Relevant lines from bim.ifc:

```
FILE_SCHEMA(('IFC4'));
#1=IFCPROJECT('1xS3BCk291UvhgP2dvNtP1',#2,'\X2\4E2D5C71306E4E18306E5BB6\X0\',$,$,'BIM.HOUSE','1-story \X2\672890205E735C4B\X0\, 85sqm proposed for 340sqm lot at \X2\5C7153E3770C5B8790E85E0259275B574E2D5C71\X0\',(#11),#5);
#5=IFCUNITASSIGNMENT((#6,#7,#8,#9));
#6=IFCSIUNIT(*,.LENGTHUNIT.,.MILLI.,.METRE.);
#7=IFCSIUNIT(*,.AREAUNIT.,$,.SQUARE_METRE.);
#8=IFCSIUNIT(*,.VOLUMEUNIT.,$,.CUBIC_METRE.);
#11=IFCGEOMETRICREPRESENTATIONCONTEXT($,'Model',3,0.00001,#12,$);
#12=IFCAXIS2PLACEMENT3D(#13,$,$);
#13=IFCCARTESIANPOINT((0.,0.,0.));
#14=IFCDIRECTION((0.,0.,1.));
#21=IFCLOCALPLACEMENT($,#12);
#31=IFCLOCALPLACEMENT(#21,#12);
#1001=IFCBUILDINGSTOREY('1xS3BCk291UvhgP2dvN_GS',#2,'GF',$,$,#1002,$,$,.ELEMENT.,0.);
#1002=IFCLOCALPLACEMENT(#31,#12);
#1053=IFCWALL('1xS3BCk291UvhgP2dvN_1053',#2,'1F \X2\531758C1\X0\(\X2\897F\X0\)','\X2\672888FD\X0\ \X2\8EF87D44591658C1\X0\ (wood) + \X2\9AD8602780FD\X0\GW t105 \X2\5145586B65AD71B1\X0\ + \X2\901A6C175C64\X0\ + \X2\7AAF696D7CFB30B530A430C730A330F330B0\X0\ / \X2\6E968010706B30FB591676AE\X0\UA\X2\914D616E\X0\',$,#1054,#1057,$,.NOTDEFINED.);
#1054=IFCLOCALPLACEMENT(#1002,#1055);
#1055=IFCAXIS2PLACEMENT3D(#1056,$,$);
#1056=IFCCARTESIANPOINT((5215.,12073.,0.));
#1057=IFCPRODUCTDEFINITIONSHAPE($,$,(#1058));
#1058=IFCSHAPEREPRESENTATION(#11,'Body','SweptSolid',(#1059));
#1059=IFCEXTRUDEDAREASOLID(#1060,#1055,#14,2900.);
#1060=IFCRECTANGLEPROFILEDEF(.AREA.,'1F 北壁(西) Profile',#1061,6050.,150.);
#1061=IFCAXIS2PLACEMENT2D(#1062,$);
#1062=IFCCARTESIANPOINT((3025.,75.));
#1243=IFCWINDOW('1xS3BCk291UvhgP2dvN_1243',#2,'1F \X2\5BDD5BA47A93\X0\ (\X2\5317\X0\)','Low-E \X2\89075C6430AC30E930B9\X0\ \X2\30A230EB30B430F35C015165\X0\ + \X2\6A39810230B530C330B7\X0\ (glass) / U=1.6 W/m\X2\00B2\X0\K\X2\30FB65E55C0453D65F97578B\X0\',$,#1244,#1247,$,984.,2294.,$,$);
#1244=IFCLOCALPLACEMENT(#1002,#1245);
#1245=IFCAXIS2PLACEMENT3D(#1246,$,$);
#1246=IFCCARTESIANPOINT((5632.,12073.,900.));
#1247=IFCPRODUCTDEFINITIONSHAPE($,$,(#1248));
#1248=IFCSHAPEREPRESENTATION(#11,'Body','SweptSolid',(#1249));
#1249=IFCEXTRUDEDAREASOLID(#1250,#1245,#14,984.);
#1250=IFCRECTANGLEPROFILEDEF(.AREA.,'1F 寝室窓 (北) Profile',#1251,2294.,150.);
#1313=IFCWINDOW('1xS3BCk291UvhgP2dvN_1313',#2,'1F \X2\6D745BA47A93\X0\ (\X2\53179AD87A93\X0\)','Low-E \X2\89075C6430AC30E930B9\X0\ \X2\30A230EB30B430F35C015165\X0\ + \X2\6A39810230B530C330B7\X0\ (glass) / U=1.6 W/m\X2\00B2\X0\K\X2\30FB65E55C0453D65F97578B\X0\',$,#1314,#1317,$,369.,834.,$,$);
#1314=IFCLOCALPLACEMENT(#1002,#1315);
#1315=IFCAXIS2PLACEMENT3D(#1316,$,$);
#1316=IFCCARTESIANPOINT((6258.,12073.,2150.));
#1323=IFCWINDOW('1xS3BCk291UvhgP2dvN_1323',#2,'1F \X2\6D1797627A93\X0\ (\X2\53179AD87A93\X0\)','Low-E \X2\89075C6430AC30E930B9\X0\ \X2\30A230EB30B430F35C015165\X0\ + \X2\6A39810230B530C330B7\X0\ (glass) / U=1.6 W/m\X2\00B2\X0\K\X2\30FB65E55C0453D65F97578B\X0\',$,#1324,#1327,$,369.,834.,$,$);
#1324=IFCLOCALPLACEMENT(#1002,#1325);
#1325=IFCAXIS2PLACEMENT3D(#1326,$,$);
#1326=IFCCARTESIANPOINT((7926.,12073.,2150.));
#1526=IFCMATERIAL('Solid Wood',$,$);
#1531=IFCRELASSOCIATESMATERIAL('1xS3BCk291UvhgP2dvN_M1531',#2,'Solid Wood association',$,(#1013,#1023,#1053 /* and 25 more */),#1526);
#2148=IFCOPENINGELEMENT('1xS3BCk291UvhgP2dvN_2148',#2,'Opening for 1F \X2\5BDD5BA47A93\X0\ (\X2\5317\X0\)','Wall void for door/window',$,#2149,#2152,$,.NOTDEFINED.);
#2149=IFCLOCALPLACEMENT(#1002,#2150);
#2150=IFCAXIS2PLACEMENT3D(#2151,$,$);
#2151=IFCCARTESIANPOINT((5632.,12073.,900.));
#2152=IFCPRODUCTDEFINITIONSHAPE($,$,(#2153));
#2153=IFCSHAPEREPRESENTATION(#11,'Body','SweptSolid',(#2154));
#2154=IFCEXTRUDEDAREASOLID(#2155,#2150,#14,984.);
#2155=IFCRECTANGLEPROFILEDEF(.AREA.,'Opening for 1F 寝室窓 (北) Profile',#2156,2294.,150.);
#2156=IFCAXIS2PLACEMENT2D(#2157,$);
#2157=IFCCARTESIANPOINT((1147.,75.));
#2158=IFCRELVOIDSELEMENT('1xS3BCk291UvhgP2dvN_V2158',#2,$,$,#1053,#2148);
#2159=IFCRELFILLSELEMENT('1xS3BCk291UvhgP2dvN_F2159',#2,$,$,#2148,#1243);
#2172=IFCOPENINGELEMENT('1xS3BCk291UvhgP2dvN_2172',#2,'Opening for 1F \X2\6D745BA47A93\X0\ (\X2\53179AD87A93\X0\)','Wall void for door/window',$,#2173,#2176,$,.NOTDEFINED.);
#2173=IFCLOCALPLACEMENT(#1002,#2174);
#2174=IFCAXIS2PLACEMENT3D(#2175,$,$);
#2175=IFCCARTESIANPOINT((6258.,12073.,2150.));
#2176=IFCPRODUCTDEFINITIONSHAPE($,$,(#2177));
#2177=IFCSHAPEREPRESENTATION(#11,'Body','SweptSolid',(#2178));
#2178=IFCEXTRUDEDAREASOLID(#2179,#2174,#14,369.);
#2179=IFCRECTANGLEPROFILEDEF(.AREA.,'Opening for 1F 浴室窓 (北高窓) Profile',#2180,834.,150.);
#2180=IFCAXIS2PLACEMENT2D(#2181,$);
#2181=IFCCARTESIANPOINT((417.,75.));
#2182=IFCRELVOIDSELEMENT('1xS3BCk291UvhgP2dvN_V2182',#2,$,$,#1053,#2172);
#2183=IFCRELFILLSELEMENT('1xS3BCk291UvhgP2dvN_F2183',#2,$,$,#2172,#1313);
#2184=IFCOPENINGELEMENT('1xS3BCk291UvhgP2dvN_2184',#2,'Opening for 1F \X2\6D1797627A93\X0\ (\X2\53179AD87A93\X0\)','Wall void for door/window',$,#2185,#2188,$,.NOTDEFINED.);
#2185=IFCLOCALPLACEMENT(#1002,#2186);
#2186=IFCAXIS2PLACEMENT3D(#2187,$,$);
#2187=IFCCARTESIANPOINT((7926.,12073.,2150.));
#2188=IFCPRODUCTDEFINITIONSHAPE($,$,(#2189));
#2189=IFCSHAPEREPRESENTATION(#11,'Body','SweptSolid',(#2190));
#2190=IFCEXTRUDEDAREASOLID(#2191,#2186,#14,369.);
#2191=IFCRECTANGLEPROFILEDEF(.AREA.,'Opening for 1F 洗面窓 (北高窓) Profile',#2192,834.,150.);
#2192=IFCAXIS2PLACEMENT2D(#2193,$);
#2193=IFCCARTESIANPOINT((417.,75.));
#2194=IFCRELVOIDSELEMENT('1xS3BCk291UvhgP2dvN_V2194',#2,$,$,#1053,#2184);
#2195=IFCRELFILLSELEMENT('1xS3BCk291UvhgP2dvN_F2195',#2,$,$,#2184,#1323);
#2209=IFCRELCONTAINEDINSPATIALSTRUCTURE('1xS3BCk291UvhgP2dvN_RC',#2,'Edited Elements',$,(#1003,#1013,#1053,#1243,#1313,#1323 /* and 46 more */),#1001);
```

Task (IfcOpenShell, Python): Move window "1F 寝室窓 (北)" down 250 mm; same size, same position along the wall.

```python
import numpy as np
import ifcopenshell
import ifcopenshell.api.geometry
import ifcopenshell.util.placement
import ifcopenshell.util.unit

model = ifcopenshell.open("bim.ifc")
unit_scale = ifcopenshell.util.unit.calculate_unit_scale(model)

window = model.by_guid("1xS3BCk291UvhgP2dvN_1243")
opening = window.FillsVoids[0].RelatingOpeningElement
dz = -0.25 / unit_scale

shift = np.array([0.0, 0.0, dz])
# The window is not placed relative to its opening, so move both.
for product in (opening, window):
    matrix = ifcopenshell.util.placement.get_local_placement(product.ObjectPlacement)
    matrix[:3, 3] += shift
    ifcopenshell.api.geometry.edit_object_placement(model, product=product, matrix=matrix, is_si=False)

print(f"moved by {dz * unit_scale:+.3f} m")

model.write("bim-out.ifc")
```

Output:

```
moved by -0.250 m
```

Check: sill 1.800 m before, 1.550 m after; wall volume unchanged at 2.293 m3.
